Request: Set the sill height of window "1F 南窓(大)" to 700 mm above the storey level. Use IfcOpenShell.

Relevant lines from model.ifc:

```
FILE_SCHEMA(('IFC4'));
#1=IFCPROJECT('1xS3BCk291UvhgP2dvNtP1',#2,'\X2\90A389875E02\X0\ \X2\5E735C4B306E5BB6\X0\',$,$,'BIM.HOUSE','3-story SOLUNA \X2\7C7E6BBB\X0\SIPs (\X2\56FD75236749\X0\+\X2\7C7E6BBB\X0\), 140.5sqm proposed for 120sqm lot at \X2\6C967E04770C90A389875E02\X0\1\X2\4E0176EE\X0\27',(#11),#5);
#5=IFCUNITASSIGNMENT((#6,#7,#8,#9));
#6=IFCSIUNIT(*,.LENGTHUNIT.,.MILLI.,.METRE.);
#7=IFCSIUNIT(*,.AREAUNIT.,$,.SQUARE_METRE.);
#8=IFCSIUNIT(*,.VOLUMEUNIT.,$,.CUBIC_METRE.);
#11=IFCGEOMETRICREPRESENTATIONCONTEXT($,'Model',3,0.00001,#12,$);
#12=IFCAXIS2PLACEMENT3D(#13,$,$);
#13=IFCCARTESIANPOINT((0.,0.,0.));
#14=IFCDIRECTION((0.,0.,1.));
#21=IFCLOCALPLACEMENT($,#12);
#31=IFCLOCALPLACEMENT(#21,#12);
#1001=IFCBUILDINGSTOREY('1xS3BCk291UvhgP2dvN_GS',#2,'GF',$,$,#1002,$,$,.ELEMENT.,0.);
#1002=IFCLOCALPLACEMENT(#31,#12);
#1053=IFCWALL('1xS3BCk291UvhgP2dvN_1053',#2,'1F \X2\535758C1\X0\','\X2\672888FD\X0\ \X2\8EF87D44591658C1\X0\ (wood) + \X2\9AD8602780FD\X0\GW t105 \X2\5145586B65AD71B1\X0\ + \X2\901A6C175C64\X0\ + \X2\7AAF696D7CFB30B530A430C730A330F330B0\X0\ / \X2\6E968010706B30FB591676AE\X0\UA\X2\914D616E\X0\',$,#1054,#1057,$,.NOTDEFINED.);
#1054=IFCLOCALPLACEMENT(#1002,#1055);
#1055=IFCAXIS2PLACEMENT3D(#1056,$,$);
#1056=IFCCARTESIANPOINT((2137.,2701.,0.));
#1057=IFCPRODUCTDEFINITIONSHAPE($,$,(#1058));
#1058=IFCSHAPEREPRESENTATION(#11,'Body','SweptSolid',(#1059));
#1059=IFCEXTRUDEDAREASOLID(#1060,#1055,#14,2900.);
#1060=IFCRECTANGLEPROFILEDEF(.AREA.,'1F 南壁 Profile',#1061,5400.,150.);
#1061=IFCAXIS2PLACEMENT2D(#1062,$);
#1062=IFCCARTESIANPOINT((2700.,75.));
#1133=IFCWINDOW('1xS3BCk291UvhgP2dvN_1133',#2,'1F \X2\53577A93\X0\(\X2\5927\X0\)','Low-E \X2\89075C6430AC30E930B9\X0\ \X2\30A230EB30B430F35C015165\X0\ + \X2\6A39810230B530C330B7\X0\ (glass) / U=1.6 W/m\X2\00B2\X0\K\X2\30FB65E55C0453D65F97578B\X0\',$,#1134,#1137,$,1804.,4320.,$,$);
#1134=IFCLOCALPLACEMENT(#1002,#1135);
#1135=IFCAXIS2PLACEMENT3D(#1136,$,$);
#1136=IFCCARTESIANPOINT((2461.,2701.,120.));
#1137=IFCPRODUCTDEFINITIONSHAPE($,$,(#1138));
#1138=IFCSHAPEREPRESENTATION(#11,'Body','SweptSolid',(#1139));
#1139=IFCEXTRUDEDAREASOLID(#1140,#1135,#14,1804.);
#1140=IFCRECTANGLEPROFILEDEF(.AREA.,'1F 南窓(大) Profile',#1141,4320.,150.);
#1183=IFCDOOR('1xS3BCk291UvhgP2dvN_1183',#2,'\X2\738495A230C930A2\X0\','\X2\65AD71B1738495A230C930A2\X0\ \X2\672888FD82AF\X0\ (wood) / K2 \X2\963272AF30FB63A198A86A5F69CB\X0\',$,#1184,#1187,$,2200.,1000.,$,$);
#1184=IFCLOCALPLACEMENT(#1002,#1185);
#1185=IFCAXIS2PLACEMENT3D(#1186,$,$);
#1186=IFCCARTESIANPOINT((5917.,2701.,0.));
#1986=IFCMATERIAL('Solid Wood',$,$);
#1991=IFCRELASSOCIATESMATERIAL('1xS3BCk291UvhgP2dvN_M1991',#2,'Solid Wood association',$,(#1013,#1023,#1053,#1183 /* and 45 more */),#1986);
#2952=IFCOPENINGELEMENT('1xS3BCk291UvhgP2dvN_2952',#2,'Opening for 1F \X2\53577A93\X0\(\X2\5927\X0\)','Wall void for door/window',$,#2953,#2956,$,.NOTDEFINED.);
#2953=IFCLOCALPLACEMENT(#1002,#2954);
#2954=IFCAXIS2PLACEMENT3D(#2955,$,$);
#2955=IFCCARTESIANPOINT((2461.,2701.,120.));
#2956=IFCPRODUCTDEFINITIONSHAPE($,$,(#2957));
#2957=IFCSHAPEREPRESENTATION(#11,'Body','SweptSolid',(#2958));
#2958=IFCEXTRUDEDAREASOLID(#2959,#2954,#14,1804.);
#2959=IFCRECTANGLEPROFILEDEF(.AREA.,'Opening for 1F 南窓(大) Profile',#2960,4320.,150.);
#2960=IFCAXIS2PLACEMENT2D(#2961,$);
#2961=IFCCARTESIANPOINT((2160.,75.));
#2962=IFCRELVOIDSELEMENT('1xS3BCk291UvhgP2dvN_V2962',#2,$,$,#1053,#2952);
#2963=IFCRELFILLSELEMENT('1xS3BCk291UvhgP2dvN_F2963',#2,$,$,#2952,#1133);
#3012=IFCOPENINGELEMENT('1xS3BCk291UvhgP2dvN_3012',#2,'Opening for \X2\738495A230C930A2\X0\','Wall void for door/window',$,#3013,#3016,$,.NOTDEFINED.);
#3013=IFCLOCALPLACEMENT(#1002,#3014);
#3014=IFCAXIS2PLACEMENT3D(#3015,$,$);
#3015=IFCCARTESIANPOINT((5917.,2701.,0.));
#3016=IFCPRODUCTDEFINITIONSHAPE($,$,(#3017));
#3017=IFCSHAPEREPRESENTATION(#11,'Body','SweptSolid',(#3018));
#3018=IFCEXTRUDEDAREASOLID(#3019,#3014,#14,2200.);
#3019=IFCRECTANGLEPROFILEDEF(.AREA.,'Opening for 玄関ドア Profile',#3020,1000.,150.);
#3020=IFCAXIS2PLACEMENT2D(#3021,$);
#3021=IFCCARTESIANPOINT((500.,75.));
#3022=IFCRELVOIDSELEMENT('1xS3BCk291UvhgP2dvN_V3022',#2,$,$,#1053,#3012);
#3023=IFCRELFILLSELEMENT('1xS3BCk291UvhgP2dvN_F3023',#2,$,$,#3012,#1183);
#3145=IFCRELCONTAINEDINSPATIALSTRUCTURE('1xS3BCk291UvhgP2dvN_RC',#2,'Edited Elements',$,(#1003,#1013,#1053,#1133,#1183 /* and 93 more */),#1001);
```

```python
import numpy as np
import ifcopenshell
import ifcopenshell.api.geometry
import ifcopenshell.geom
import ifcopenshell.util.element
import ifcopenshell.util.placement
import ifcopenshell.util.shape
import ifcopenshell.util.unit

model = ifcopenshell.open("model.ifc")
unit_scale = ifcopenshell.util.unit.calculate_unit_scale(model)

window = model.by_guid("1xS3BCk291UvhgP2dvN_1133")
opening = window.FillsVoids[0].RelatingOpeningElement
storey = ifcopenshell.util.element.get_container(window, ifc_class="IfcBuildingStorey")
level = ifcopenshell.util.placement.get_local_placement(storey.ObjectPlacement)[2, 3]

# The opening's origin need not be at the sill, so measure its lowest point.
shape = ifcopenshell.geom.create_shape(ifcopenshell.geom.settings(), opening)
bottom = ifcopenshell.util.shape.get_shape_bottom_elevation(shape, shape.geometry) / unit_scale
dz = level + 700.0 - bottom

shift = np.array([0.0, 0.0, dz])
# The window is not placed relative to its opening, so move both.
for product in (opening, window):
    matrix = ifcopenshell.util.placement.get_local_placement(product.ObjectPlacement)
    matrix[:3, 3] += shift
    ifcopenshell.api.geometry.edit_object_placement(model, product=product, matrix=matrix, is_si=False)

print(f"moved by {dz * unit_scale:+.3f} m")

model.write("model_v2.ifc")
```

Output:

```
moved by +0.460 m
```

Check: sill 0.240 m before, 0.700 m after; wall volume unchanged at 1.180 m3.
